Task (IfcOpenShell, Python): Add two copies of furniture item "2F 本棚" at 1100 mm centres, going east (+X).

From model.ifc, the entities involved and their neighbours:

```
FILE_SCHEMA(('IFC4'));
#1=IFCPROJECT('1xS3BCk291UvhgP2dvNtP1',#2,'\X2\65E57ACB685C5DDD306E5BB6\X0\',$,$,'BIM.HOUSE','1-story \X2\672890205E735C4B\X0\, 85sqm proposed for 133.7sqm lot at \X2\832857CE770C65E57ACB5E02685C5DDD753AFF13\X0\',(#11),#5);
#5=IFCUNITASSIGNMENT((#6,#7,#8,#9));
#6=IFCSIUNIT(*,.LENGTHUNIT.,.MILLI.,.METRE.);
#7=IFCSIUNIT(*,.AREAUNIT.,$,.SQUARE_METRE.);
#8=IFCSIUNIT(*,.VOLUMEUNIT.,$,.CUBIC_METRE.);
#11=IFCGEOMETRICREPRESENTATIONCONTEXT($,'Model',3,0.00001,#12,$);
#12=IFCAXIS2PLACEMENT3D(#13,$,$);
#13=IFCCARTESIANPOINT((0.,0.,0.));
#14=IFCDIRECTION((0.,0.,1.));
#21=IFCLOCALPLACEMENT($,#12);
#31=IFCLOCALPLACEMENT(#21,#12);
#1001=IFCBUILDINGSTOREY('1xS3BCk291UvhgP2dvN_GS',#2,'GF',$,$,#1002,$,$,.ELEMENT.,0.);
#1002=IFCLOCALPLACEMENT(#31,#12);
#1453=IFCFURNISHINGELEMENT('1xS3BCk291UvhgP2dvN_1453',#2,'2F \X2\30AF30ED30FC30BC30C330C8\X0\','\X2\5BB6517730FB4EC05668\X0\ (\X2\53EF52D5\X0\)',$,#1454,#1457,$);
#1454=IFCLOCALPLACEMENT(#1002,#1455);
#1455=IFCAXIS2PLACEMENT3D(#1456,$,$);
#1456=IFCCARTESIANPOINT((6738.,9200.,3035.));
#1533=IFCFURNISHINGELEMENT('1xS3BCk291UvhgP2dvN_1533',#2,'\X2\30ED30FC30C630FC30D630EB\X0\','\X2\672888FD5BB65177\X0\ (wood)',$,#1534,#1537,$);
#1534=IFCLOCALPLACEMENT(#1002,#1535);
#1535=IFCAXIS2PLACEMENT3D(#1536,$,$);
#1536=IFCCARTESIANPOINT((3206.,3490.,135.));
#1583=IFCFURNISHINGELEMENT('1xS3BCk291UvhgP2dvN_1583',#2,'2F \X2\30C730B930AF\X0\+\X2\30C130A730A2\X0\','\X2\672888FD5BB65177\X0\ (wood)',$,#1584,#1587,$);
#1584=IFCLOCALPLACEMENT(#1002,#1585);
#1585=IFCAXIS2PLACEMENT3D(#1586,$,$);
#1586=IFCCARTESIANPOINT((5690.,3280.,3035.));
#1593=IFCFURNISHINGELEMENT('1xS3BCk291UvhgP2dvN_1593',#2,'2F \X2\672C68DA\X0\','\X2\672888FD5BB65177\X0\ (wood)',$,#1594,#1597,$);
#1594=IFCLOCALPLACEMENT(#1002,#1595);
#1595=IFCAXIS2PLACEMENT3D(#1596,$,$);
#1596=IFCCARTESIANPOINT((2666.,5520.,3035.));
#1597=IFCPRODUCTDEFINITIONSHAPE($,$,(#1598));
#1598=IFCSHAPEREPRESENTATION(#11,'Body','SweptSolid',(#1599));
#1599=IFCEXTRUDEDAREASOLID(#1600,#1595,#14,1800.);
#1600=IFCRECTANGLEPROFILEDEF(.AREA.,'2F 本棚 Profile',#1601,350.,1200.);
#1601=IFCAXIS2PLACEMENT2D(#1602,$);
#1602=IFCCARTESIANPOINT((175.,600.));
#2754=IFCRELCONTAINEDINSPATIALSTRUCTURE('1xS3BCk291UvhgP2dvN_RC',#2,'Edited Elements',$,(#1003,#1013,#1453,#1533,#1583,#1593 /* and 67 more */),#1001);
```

```python
import numpy as np
import ifcopenshell
import ifcopenshell.api.geometry
import ifcopenshell.api.root
import ifcopenshell.util.element
import ifcopenshell.util.placement
import ifcopenshell.util.unit

model = ifcopenshell.open("model.ifc")
unit_scale = ifcopenshell.util.unit.calculate_unit_scale(model)


def reuse_history(source, copy):
    """copy_class also copies each property set's owner history, people and application; keep the originals."""
    for rel in copy.IsDefinedBy:
        if rel.is_a("IfcRelDefinesByProperties") and (history := rel.RelatingPropertyDefinition.OwnerHistory):
            rel.RelatingPropertyDefinition.OwnerHistory = source.OwnerHistory
            ifcopenshell.util.element.remove_deep2(model, history)


source = model.by_id(1593)
base = ifcopenshell.util.placement.get_local_placement(source.ObjectPlacement)
step = np.array([1.0, 0.0, 0.0]) * 1.1 / unit_scale

for i in range(1, 3):
    copy = ifcopenshell.api.root.copy_class(model, product=source)
    copy.Representation = ifcopenshell.util.element.copy_deep(
        model, source.Representation, exclude=["IfcGeometricRepresentationContext", "IfcRepresentationMap"]
    )
    reuse_history(source, copy)
    matrix = base.copy()
    matrix[:3, 3] += i * step
    print("added at", matrix[:3, 3].round(3) + 0.0)
    ifcopenshell.api.geometry.edit_object_placement(model, product=copy, matrix=matrix, is_si=False)

model.write("model_v2.ifc")
```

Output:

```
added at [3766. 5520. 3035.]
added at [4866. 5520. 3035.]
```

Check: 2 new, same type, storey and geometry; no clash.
